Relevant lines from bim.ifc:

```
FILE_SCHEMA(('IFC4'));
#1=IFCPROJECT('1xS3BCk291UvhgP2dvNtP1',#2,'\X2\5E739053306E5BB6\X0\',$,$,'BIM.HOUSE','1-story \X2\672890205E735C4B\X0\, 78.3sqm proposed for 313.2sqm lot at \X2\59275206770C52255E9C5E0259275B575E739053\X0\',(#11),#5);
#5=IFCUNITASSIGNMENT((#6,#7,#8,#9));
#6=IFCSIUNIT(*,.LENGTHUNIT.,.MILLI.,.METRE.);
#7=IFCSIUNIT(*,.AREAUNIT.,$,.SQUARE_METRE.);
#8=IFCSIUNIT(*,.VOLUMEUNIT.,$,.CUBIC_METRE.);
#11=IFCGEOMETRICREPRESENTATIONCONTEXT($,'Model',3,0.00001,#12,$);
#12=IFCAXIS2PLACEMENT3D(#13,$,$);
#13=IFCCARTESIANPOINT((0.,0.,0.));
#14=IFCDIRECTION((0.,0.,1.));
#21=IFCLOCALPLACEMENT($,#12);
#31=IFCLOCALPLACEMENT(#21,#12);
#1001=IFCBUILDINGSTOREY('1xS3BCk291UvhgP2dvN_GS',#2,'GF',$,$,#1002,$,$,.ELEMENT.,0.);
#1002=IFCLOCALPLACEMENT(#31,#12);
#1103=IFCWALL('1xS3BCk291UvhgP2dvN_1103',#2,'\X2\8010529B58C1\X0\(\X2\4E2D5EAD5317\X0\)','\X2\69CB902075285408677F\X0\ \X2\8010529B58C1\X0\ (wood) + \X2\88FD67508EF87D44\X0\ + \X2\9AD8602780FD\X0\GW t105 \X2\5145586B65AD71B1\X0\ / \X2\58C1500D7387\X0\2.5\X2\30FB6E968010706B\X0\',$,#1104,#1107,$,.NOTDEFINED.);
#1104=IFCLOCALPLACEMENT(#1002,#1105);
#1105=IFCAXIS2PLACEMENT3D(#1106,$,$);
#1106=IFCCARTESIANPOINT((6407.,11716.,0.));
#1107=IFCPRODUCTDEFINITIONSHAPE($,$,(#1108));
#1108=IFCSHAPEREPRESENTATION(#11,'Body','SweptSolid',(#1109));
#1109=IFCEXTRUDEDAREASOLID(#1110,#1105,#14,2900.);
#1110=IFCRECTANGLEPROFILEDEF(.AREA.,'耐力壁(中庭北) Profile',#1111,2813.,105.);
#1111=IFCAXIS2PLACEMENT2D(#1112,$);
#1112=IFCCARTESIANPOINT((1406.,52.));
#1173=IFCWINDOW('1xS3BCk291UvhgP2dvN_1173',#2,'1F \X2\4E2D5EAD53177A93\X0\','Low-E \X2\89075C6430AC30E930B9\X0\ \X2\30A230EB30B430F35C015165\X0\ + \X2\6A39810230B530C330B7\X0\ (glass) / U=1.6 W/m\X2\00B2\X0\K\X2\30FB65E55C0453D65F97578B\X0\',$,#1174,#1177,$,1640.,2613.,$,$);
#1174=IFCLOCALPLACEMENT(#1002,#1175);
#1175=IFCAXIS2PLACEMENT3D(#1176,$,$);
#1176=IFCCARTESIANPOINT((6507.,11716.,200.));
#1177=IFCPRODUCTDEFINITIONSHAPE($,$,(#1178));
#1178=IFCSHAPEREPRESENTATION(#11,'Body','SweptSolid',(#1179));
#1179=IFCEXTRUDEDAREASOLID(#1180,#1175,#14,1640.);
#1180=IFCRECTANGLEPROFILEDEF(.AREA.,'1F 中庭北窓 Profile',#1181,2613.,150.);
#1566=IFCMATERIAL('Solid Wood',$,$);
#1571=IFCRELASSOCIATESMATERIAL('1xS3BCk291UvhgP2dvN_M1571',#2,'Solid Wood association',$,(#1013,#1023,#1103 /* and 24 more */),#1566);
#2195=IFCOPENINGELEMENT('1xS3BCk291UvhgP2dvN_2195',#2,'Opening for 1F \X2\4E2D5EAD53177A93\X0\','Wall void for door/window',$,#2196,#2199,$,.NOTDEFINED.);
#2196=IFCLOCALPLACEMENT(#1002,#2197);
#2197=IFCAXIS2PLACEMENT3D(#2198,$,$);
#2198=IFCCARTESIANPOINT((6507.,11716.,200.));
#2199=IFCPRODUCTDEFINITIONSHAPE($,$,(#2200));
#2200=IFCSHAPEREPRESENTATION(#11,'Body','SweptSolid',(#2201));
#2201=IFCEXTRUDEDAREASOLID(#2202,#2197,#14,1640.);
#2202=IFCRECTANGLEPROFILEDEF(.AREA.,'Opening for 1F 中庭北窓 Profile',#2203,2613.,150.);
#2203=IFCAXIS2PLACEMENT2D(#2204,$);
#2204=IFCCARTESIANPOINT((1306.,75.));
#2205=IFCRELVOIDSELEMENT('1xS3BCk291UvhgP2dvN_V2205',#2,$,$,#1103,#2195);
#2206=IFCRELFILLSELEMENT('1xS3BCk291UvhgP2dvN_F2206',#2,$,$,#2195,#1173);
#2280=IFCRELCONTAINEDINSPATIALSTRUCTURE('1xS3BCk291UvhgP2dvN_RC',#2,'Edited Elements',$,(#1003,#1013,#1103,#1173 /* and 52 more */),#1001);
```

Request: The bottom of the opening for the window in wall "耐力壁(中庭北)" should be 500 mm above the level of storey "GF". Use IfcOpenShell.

```python
import numpy as np
import ifcopenshell
import ifcopenshell.api.geometry
import ifcopenshell.geom
import ifcopenshell.util.element
import ifcopenshell.util.placement
import ifcopenshell.util.shape
import ifcopenshell.util.unit

model = ifcopenshell.open("bim.ifc")
unit_scale = ifcopenshell.util.unit.calculate_unit_scale(model)

window = model.by_guid("1xS3BCk291UvhgP2dvN_1173")
opening = window.FillsVoids[0].RelatingOpeningElement
storey = ifcopenshell.util.element.get_container(window, ifc_class="IfcBuildingStorey")
level = ifcopenshell.util.placement.get_local_placement(storey.ObjectPlacement)[2, 3]

# The opening's origin need not be at the sill, so measure its lowest point.
shape = ifcopenshell.geom.create_shape(ifcopenshell.geom.settings(), opening)
bottom = ifcopenshell.util.shape.get_shape_bottom_elevation(shape, shape.geometry) / unit_scale
dz = level + 0.5 / unit_scale - bottom

shift = np.array([0.0, 0.0, dz])
# The window is not placed relative to its opening, so move both.
for product in (opening, window):
    matrix = ifcopenshell.util.placement.get_local_placement(product.ObjectPlacement)
    matrix[:3, 3] += shift
    ifcopenshell.api.geometry.edit_object_placement(model, product=product, matrix=matrix, is_si=False)

print(f"moved by {dz * unit_scale:+.3f} m")

model.write("bim_v2.ifc")
```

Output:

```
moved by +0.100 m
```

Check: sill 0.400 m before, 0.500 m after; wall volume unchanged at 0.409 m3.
